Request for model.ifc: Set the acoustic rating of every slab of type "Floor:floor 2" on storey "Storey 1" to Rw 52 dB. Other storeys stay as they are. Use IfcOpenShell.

First a look at what the model holds.

```python
import ifcopenshell
import ifcopenshell.util.element

model = ifcopenshell.open("model.ifc")
print(model.schema)
storey = next(s for s in model.by_type("IfcBuildingStorey") if s.Name == "Storey 1")
slabs = [e for e in ifcopenshell.util.element.get_decomposition(storey) if e.is_a("IfcSlab")]
seen = {}
for e in slabs:
    element_type = ifcopenshell.util.element.get_type(e)
    key = (element_type.Name if element_type != e and element_type else None, ifcopenshell.util.element.get_pset(e, "Pset_SlabCommon", "AcousticRating"))
    seen[key] = seen.get(key, 0) + 1
for (name, value), count in sorted(seen.items(), key=str):
    print(count, "x", name, "|", value)
```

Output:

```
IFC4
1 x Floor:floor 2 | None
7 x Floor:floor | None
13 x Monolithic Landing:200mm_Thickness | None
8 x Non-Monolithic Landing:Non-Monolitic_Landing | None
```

```python
import ifcopenshell
import ifcopenshell.api.pset
import ifcopenshell.util.element

model = ifcopenshell.open("model.ifc")

storey = next(s for s in model.by_type("IfcBuildingStorey") if s.Name == "Storey 1")
slabs = [e for e in ifcopenshell.util.element.get_decomposition(storey) if e.is_a("IfcSlab")]

count = 0
for e in slabs:
    element_type = ifcopenshell.util.element.get_type(e)
    if element_type in (None, e) or element_type.Name != "Floor:floor 2":
        continue
    # add_pset returns the element's existing set when there is one.
    pset = ifcopenshell.api.pset.add_pset(model, product=e, name="Pset_SlabCommon")
    ifcopenshell.api.pset.edit_pset(model, pset=pset, properties={"AcousticRating": "Rw 52 dB"})
    count += 1

print(count, "slabs updated")

model.write("model_edited.ifc")
```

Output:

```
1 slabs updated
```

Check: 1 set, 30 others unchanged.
